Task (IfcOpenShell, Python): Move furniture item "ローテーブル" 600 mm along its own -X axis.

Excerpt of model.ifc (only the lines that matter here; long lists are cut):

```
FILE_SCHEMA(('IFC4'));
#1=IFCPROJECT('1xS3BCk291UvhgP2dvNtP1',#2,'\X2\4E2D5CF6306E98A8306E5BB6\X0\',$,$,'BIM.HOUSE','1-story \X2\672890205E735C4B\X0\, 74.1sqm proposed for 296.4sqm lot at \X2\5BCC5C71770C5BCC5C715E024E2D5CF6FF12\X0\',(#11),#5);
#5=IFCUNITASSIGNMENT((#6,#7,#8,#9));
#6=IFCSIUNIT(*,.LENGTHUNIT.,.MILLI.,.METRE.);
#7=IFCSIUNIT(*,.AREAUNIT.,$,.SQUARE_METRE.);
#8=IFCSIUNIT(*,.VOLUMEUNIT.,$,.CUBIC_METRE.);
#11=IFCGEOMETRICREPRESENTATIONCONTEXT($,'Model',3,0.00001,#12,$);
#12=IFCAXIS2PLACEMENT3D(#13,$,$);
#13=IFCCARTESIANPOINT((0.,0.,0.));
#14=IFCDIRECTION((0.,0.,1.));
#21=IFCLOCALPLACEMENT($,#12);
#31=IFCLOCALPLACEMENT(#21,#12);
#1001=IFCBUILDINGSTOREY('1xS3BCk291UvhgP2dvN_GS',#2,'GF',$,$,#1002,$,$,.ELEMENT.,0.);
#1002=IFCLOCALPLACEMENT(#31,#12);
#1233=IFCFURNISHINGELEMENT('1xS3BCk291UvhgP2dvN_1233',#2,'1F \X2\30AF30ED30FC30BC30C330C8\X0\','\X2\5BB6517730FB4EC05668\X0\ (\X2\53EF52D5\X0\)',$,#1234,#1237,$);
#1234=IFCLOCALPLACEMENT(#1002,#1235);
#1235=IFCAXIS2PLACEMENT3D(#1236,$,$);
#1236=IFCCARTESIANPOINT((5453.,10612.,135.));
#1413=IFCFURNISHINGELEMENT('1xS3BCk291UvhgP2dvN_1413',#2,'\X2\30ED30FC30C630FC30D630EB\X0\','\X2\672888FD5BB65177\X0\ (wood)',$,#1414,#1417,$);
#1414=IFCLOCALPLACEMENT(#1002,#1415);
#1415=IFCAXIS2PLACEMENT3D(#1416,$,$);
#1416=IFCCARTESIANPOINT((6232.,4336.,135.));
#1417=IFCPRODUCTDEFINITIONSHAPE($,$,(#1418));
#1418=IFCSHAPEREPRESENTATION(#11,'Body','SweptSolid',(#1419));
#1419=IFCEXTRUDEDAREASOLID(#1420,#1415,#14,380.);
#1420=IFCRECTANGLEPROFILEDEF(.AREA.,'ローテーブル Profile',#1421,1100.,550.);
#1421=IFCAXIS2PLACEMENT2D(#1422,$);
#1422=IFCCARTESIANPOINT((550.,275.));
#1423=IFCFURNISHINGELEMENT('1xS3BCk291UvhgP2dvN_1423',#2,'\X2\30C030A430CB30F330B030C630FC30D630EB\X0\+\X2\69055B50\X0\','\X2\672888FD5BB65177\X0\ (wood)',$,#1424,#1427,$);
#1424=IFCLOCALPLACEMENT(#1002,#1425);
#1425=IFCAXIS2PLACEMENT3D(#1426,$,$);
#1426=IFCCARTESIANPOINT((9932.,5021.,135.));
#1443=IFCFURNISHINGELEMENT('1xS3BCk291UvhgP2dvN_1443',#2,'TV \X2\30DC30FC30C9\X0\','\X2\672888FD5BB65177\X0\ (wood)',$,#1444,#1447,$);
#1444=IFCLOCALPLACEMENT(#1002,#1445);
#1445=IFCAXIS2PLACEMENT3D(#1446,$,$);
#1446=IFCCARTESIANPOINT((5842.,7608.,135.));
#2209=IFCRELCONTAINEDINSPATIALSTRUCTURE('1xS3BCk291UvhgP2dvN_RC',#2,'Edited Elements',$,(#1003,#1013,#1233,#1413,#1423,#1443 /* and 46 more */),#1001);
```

```python
import ifcopenshell
import ifcopenshell.api.geometry
import ifcopenshell.util.placement

model = ifcopenshell.open("model.ifc")

item = model.by_guid("1xS3BCk291UvhgP2dvN_1413")
matrix = ifcopenshell.util.placement.get_local_placement(item.ObjectPlacement)
matrix[:3, 3] -= matrix[:3, 0] * 600.0
ifcopenshell.api.geometry.edit_object_placement(model, product=item, matrix=matrix, is_si=False)

print(ifcopenshell.util.placement.get_local_placement(item.ObjectPlacement).round(3) + 0.0)

model.write("model_edited.ifc")
```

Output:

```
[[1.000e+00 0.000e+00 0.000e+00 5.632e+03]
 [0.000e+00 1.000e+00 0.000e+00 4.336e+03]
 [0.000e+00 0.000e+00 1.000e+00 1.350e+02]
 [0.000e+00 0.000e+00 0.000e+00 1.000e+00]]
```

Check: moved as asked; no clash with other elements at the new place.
